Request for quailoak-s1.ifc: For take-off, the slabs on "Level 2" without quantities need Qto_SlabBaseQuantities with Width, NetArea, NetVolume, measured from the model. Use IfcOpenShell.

First a look at what the model holds.

```python
import ifcopenshell
import ifcopenshell.util.element
import ifcopenshell.util.unit

model = ifcopenshell.open("quailoak-s1.ifc")
print(model.schema)
for unit_type in ("LENGTHUNIT", "AREAUNIT", "VOLUMEUNIT"):
    print(unit_type, ifcopenshell.util.unit.calculate_unit_scale(model, unit_type))
storey = next(s for s in model.by_type("IfcBuildingStorey") if s.Name == "Level 2")
slabs = [e for e in ifcopenshell.util.element.get_decomposition(storey) if e.is_a("IfcSlab")]
for e in sorted(slabs, key=lambda e: e.id()):
    print(e.id(), e.is_a(), e.Name, list(ifcopenshell.util.element.get_psets(e, qtos_only=True)), sep=" | ")
```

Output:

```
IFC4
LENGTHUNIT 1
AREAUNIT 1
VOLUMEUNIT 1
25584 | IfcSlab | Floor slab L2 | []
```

```python
import ifcopenshell
import ifcopenshell.api.pset
import ifcopenshell.geom
import ifcopenshell.util.element
import ifcopenshell.util.shape
import ifcopenshell.util.unit

model = ifcopenshell.open("quailoak-s1.ifc")
unit_scale = ifcopenshell.util.unit.calculate_unit_scale(model)
area_scale = ifcopenshell.util.unit.calculate_unit_scale(model, "AREAUNIT")
volume_scale = ifcopenshell.util.unit.calculate_unit_scale(model, "VOLUMEUNIT")
settings = ifcopenshell.geom.settings()

storey = next(s for s in model.by_type("IfcBuildingStorey") if s.Name == "Level 2")
slabs = [e for e in ifcopenshell.util.element.get_decomposition(storey) if e.is_a("IfcSlab")]

for e in sorted(slabs, key=lambda e: e.id()):
    if ifcopenshell.util.element.get_psets(e, qtos_only=True, should_inherit=False):
        continue
    # Geometry comes back in metres, in the element's own axes.
    shape = ifcopenshell.geom.create_shape(settings, e)
    values = {
        "Width": ifcopenshell.util.shape.get_z(shape.geometry) / unit_scale,
        "NetArea": ifcopenshell.util.shape.get_footprint_area(shape.geometry) / area_scale,
        "NetVolume": ifcopenshell.util.shape.get_volume(shape.geometry) / volume_scale,
    }
    qto = ifcopenshell.api.pset.add_qto(model, product=e, name="Qto_SlabBaseQuantities")
    ifcopenshell.api.pset.edit_qto(model, qto=qto, properties=values)
    print(e.id(), {k: round(v, 3) for k, v in values.items()})

model.write("quailoak-s1_v2.ifc")
```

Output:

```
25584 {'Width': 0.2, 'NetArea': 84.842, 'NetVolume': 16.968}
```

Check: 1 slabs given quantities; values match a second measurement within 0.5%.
